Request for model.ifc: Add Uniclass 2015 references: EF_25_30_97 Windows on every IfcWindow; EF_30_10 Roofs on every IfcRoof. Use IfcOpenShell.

First a look at what the model holds.

```python
import ifcopenshell

model = ifcopenshell.open("model.ifc")
print(model.schema)
print("classifications:", [c.Name for c in model.by_type("IfcClassification")])
for ifc_class in ("IfcDoor", "IfcRoof", "IfcStair", "IfcWall", "IfcWindow"):
    print(ifc_class, len(model.by_type(ifc_class)))
```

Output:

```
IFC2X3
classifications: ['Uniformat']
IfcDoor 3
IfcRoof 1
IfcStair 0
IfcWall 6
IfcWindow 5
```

```python
import ifcopenshell
import ifcopenshell.api.classification

model = ifcopenshell.open("model.ifc")

# IFC2X3 requires Source and Edition and has no link from the project to the system.
system = model.create_entity("IfcClassification", Source="NBS", Edition="2015", Name="Uniclass 2015")

codes = {
    "IfcWindow": ("EF_25_30_97", "Windows"),
    "IfcRoof": ("EF_30_10", "Roofs"),
}
for ifc_class, (code, name) in codes.items():
    products = model.by_type(ifc_class)
    ifcopenshell.api.classification.add_reference(
        model, products=products, classification=system, identification=code, name=name
    )
    print(code, len(products))

model.write("model_updated.ifc")
```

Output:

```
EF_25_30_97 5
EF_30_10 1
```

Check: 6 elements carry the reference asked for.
